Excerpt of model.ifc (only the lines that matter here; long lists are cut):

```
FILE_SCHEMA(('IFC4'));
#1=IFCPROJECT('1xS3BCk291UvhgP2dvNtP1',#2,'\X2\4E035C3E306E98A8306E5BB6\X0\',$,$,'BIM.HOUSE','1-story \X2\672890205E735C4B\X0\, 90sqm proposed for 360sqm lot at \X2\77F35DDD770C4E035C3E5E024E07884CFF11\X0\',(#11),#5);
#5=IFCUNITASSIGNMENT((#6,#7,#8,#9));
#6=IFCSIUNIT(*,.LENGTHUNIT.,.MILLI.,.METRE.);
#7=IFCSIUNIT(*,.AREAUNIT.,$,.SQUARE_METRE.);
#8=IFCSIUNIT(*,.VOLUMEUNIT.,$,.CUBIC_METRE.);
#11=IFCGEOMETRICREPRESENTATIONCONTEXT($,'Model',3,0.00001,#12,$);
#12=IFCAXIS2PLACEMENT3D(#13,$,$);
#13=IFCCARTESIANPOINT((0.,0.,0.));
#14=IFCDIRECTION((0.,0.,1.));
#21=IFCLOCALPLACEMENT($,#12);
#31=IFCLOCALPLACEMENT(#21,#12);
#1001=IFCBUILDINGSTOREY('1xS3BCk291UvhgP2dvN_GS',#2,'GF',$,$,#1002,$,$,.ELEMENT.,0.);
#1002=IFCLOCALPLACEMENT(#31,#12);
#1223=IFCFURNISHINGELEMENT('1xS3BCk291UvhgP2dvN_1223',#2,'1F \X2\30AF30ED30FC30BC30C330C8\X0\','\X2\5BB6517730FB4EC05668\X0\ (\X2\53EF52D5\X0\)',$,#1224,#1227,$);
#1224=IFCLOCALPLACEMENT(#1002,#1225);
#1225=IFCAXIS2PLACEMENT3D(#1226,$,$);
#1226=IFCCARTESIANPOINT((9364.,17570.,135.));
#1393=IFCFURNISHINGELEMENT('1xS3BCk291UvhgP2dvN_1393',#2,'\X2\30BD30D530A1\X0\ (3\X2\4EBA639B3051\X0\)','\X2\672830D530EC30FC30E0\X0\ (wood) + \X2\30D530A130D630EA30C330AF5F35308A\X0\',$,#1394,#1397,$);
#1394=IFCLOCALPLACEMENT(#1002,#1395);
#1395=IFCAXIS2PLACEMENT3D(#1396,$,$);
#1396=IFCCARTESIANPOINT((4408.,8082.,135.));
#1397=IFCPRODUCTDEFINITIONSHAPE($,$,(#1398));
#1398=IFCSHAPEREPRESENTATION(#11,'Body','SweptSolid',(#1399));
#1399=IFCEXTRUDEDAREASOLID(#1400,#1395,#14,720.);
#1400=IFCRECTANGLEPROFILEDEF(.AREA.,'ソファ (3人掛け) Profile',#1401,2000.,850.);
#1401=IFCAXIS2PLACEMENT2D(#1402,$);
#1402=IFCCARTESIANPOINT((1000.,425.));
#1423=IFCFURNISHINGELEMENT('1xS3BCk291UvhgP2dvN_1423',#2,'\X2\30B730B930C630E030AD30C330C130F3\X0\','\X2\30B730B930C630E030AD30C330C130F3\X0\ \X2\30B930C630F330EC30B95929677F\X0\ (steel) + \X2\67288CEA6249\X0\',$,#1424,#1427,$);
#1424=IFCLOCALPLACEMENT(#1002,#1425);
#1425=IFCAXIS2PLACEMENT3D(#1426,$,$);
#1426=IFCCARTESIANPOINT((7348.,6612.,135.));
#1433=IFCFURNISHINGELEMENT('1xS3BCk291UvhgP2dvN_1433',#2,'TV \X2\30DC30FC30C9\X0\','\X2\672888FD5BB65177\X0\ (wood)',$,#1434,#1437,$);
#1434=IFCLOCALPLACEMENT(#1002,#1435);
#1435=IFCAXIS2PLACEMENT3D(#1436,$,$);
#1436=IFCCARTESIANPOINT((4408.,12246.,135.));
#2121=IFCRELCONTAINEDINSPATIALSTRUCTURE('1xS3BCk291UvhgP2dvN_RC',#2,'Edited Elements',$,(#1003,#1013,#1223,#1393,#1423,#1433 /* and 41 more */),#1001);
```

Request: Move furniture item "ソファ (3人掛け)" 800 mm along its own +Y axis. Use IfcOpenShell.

```python
import ifcopenshell
import ifcopenshell.api.geometry
import ifcopenshell.util.placement

model = ifcopenshell.open("model.ifc")

item = model.by_guid("1xS3BCk291UvhgP2dvN_1393")
matrix = ifcopenshell.util.placement.get_local_placement(item.ObjectPlacement)
matrix[:3, 3] += matrix[:3, 1] * 800.0
ifcopenshell.api.geometry.edit_object_placement(model, product=item, matrix=matrix, is_si=False)

print(ifcopenshell.util.placement.get_local_placement(item.ObjectPlacement).round(3) + 0.0)

model.write("model_updated.ifc")
```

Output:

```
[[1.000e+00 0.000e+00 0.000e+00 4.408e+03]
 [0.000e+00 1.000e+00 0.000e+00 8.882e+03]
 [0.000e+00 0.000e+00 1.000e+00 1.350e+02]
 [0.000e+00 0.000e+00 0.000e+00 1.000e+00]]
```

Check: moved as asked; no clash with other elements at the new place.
